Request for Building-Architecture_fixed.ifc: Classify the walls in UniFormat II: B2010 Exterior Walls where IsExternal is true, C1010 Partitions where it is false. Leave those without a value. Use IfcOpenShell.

First a look at what the model holds.

```python
import ifcopenshell
import ifcopenshell.util.element

model = ifcopenshell.open("Building-Architecture_fixed.ifc")
print(model.schema)
print("classifications:", [c.Name for c in model.by_type("IfcClassification")])
values = [ifcopenshell.util.element.get_pset(e, "Pset_WallCommon", "IsExternal") for e in model.by_type("IfcWall")]
for value in (True, False, None):
    print("IsExternal", value, values.count(value))
```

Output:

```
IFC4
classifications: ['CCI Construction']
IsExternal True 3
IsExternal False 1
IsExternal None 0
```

```python
import ifcopenshell
import ifcopenshell.api.classification
import ifcopenshell.util.element

model = ifcopenshell.open("Building-Architecture_fixed.ifc")

system = ifcopenshell.api.classification.add_classification(model, classification="UniFormat II")

walls = model.by_type("IfcWall")
external = {e: ifcopenshell.util.element.get_pset(e, "Pset_WallCommon", "IsExternal") for e in walls}
for flag, code, name in ((True, "B2010", "Exterior Walls"), (False, "C1010", "Partitions")):
    products = [e for e in walls if external[e] is flag]
    ifcopenshell.api.classification.add_reference(
        model, products=products, classification=system, identification=code, name=name
    )
    print(code, len(products))

model.write("Building-Architecture_fixed_edited.ifc")
```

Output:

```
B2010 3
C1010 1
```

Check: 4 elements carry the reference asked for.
